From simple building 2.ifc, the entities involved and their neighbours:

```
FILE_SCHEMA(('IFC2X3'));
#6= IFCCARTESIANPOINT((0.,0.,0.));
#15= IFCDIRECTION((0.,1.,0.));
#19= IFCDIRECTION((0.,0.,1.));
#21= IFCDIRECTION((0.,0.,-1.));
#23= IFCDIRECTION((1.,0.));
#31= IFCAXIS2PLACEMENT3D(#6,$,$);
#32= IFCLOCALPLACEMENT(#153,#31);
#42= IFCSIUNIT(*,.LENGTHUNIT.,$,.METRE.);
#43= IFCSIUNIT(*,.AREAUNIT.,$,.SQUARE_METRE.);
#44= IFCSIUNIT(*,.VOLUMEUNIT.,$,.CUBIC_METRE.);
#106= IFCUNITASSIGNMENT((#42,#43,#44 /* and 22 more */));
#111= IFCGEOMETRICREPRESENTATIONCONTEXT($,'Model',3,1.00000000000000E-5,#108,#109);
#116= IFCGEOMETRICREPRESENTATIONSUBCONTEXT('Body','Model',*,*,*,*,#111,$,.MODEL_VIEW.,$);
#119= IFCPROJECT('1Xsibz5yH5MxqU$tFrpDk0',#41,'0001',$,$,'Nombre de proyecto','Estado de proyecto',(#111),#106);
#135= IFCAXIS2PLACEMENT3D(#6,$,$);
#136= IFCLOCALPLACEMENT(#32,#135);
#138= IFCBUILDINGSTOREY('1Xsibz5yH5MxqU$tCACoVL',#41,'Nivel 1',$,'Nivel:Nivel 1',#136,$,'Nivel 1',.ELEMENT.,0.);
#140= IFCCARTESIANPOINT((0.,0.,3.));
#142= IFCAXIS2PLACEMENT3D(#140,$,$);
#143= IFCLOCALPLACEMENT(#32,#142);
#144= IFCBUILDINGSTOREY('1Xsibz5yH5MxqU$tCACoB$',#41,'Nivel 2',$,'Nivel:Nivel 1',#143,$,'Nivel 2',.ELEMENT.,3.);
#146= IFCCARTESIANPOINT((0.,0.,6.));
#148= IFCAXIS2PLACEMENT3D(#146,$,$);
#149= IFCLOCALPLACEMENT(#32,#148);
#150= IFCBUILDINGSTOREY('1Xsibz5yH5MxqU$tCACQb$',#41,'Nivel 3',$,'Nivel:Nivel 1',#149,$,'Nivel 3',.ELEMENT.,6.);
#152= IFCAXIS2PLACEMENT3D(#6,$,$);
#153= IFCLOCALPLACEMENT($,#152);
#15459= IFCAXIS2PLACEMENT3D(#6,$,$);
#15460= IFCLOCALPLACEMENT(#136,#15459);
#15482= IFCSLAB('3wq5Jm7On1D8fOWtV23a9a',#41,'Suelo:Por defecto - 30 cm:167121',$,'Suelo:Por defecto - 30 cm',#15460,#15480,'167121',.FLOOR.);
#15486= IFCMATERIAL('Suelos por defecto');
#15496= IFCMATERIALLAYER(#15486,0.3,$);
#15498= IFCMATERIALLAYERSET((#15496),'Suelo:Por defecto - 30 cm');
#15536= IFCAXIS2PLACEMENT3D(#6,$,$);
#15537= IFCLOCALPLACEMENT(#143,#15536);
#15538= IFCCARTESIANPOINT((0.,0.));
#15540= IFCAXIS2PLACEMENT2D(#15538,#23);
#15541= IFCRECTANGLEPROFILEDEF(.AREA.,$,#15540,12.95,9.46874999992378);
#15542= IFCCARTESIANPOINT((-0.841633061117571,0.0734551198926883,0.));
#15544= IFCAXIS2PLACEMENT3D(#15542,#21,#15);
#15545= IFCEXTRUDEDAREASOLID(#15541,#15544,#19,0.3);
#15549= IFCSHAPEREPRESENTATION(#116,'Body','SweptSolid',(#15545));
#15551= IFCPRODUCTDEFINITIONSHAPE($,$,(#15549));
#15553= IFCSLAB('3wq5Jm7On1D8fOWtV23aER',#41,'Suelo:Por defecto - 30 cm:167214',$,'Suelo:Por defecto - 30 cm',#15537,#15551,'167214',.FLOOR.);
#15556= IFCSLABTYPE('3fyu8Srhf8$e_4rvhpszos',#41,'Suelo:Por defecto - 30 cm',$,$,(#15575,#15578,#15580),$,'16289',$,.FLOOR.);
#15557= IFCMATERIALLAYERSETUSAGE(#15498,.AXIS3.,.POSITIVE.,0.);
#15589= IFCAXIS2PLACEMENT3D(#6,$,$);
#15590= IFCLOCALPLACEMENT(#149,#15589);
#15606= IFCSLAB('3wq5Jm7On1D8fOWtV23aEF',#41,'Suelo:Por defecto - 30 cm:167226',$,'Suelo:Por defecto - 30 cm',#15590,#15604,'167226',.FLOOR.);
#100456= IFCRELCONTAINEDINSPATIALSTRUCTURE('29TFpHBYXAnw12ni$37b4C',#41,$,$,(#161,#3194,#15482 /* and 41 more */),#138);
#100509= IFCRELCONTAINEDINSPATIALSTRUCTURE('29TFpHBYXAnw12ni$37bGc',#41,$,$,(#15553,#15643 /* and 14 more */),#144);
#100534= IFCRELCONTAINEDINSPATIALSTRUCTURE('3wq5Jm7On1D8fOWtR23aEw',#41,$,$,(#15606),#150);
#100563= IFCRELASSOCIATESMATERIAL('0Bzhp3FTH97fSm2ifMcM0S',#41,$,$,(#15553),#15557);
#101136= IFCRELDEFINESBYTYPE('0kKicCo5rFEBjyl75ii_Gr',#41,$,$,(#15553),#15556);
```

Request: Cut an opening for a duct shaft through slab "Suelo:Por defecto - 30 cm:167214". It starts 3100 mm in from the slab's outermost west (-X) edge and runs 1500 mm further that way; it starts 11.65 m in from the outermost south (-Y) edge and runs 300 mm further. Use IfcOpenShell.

```python
import numpy as np
import ifcopenshell
import ifcopenshell.api.feature
import ifcopenshell.api.geometry
import ifcopenshell.api.root
import ifcopenshell.geom
import ifcopenshell.util.placement
import ifcopenshell.util.representation
import ifcopenshell.util.shape
import ifcopenshell.util.unit

model = ifcopenshell.open("simple building 2.ifc")
unit_scale = ifcopenshell.util.unit.calculate_unit_scale(model)
settings = ifcopenshell.geom.settings()


def volume(element):
    """Net volume in cubic metres, openings subtracted."""
    shape = ifcopenshell.geom.create_shape(settings, element)
    return ifcopenshell.util.shape.get_volume(shape.geometry)


slab = model.by_id(15553)
before = volume(slab)

# Extent in the slab's own axes, in metres. The edges named are its -X and -Y sides.
slab_shape = ifcopenshell.geom.create_shape(settings, slab)
vertices = ifcopenshell.util.shape.get_vertices(slab_shape.geometry)
x_min, y_min, bottom = vertices.min(axis=0)
top = vertices[:, 2].max()

opening = ifcopenshell.api.root.create_entity(model, ifc_class="IfcOpeningElement", name="Duct shaft opening")
context = ifcopenshell.util.representation.get_context(model, "Model", "Body", "MODEL_VIEW")
width, depth = 1.5, 0.3
outline = [(0.0, 0.0), (width, 0.0), (width, depth), (0.0, depth), (0.0, 0.0)]
# Overshoot both faces by 50 mm so the cut is clean.
shape = ifcopenshell.api.geometry.add_slab_representation(
    model, context=context, depth=top - bottom + 0.1, polyline=outline
)
ifcopenshell.api.geometry.assign_representation(model, product=opening, representation=shape)

matrix = ifcopenshell.util.placement.get_local_placement(slab.ObjectPlacement)
matrix[:, 3] = matrix @ np.append(np.array([x_min + 3.1, y_min + 11.65, bottom - 0.05]) / unit_scale, 1.0)
ifcopenshell.api.geometry.edit_object_placement(model, product=opening, matrix=matrix, is_si=False)
ifcopenshell.api.feature.add_feature(model, feature=opening, element=slab)

after = volume(slab)

print(f"slab volume {before:.3f} -> {after:.3f} m3")

model.write("simple building 2-out.ifc")
```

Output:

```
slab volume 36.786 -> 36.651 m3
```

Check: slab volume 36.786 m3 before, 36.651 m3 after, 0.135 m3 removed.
